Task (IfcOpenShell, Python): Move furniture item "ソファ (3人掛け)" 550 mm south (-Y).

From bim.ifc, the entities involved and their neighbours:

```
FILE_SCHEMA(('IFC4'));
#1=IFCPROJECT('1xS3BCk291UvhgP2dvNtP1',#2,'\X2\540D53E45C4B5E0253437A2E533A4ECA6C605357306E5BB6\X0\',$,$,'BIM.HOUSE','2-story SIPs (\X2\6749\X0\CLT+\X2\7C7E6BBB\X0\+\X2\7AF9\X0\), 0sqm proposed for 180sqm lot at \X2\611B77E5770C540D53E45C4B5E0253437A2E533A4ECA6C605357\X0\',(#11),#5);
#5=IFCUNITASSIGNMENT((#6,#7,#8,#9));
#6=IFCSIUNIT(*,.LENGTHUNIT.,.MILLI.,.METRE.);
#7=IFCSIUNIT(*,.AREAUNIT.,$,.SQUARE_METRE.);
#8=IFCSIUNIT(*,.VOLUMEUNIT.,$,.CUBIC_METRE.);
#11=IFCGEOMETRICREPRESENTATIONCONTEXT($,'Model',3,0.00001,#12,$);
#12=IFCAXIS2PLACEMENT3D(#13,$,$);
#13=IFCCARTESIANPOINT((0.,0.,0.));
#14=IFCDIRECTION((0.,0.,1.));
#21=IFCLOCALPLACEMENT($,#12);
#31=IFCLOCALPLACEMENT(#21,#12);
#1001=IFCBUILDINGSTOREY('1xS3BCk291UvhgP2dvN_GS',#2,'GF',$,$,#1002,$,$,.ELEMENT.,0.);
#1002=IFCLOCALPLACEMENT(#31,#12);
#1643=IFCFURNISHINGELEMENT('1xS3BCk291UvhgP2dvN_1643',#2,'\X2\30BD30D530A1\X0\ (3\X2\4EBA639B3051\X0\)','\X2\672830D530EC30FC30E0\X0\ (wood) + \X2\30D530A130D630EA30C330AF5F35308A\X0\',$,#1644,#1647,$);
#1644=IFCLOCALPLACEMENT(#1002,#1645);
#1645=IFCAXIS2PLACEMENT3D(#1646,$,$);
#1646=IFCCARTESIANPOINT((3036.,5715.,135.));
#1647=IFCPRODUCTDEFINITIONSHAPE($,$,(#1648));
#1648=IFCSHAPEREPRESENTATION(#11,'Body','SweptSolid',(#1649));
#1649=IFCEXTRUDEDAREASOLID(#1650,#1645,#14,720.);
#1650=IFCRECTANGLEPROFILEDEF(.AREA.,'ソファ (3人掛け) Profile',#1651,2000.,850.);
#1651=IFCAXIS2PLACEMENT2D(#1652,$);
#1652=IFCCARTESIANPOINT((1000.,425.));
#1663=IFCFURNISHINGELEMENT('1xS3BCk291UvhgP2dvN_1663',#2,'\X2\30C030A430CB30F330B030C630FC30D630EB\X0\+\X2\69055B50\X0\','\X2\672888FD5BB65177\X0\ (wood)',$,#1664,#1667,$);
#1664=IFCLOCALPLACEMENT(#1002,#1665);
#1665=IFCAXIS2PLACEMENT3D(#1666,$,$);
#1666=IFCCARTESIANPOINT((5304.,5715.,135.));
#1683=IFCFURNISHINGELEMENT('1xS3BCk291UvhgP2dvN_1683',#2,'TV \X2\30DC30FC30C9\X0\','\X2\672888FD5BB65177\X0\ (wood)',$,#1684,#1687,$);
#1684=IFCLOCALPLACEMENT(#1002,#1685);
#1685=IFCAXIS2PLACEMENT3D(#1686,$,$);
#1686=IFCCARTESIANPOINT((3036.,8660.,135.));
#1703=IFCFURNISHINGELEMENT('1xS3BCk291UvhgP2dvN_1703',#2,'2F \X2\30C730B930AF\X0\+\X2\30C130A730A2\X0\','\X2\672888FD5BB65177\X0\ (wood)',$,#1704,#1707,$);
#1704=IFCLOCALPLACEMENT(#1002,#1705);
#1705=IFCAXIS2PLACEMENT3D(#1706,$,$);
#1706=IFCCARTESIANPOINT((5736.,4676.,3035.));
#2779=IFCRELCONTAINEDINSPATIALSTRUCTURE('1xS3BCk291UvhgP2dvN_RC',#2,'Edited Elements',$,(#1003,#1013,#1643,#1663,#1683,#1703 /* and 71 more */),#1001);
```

```python
import ifcopenshell
import ifcopenshell.api.geometry
import ifcopenshell.util.placement
import ifcopenshell.util.unit

model = ifcopenshell.open("bim.ifc")
unit_scale = ifcopenshell.util.unit.calculate_unit_scale(model)

item = model.by_guid("1xS3BCk291UvhgP2dvN_1643")
matrix = ifcopenshell.util.placement.get_local_placement(item.ObjectPlacement)
matrix[1, 3] -= 0.55 / unit_scale
ifcopenshell.api.geometry.edit_object_placement(model, product=item, matrix=matrix, is_si=False)

print(ifcopenshell.util.placement.get_local_placement(item.ObjectPlacement).round(3) + 0.0)

model.write("bim_v2.ifc")
```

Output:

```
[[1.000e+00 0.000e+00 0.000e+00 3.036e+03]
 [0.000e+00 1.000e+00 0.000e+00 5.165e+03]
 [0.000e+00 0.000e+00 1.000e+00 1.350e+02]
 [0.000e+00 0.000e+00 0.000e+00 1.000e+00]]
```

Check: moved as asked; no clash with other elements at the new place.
